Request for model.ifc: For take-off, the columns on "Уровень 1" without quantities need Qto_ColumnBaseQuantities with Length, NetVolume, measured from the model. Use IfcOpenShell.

First a look at what the model holds.

```python
import ifcopenshell
import ifcopenshell.util.element
import ifcopenshell.util.unit

model = ifcopenshell.open("model.ifc")
print(model.schema)
for unit_type in ("LENGTHUNIT", "AREAUNIT", "VOLUMEUNIT"):
    print(unit_type, ifcopenshell.util.unit.calculate_unit_scale(model, unit_type))
storey = next(s for s in model.by_type("IfcBuildingStorey") if s.Name == "Уровень 1")
columns = [e for e in ifcopenshell.util.element.get_decomposition(storey) if e.is_a("IfcColumn")]
for e in sorted(columns, key=lambda e: e.id()):
    print(e.id(), e.is_a(), e.Name, list(ifcopenshell.util.element.get_psets(e, qtos_only=True)), sep=" | ")
```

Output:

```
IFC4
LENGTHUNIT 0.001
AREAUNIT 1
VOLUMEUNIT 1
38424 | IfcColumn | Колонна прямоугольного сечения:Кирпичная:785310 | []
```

```python
import ifcopenshell
import ifcopenshell.api.pset
import ifcopenshell.geom
import ifcopenshell.util.element
import ifcopenshell.util.shape
import ifcopenshell.util.unit

model = ifcopenshell.open("model.ifc")
unit_scale = ifcopenshell.util.unit.calculate_unit_scale(model)
volume_scale = ifcopenshell.util.unit.calculate_unit_scale(model, "VOLUMEUNIT")
settings = ifcopenshell.geom.settings()

storey = next(s for s in model.by_type("IfcBuildingStorey") if s.Name == "Уровень 1")
columns = [e for e in ifcopenshell.util.element.get_decomposition(storey) if e.is_a("IfcColumn")]

for e in sorted(columns, key=lambda e: e.id()):
    if ifcopenshell.util.element.get_psets(e, qtos_only=True, should_inherit=False):
        continue
    # Geometry comes back in metres, in the element's own axes.
    shape = ifcopenshell.geom.create_shape(settings, e)
    values = {
        "Length": ifcopenshell.util.shape.get_z(shape.geometry) / unit_scale,
        "NetVolume": ifcopenshell.util.shape.get_volume(shape.geometry) / volume_scale,
    }
    qto = ifcopenshell.api.pset.add_qto(model, product=e, name="Qto_ColumnBaseQuantities")
    ifcopenshell.api.pset.edit_qto(model, qto=qto, properties=values)
    print(e.id(), {k: round(v, 3) for k, v in values.items()})

model.write("model_v2.ifc")
```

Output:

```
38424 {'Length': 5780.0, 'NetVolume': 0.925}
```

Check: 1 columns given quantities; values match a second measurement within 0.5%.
